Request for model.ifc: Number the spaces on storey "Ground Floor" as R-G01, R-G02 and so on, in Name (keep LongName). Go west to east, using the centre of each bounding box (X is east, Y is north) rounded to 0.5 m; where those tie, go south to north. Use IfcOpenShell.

First a look at what the model holds.

```python
import ifcopenshell
import ifcopenshell.util.element
import ifcopenshell.util.placement

model = ifcopenshell.open("model.ifc")
print(model.schema)
storey = next(s for s in model.by_type("IfcBuildingStorey") if s.Name == "Ground Floor")
spaces = [e for e in ifcopenshell.util.element.get_decomposition(storey) if e.is_a("IfcSpace")]
for e in sorted(spaces, key=lambda e: e.id()):
    origin = ifcopenshell.util.placement.get_local_placement(e.ObjectPlacement)[:3, 3]
    print(e.id(), e.Name, e.LongName, origin.round(2) + 0.0, sep=" | ")
```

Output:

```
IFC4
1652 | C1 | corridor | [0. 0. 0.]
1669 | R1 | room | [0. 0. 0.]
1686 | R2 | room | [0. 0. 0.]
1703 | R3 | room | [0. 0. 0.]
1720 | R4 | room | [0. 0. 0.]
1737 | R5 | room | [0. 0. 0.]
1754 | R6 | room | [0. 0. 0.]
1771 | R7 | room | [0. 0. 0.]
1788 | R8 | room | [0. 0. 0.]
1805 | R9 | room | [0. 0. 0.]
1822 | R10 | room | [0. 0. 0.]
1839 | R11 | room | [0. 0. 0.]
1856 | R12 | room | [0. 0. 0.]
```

```python
import ifcopenshell
import ifcopenshell.geom
import ifcopenshell.util.element
import ifcopenshell.util.shape

model = ifcopenshell.open("model.ifc")
settings = ifcopenshell.geom.settings()
settings.set("use-world-coords", True)


def centre(element):
    shape = ifcopenshell.geom.create_shape(settings, element)
    return ifcopenshell.util.shape.get_bbox_centroid(shape.geometry)


storey = next(s for s in model.by_type("IfcBuildingStorey") if s.Name == "Ground Floor")
spaces = [e for e in ifcopenshell.util.element.get_decomposition(storey) if e.is_a("IfcSpace")]

# Insertion points can sit at a corner or the storey origin, so sort by the geometry (in metres).
centres = {e: centre(e) for e in spaces}
spaces.sort(key=lambda e: (round(centres[e][0] / 0.5), centres[e][1]))

for i, e in enumerate(spaces, start=1):
    number = f"R-G{i:02d}"
    e.Name = number
    print(e.id(), number)

model.write("model_v2.ifc")
```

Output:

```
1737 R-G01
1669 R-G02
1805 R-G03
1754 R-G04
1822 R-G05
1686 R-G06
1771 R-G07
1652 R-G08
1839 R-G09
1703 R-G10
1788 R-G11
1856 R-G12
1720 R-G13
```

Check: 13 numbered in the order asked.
